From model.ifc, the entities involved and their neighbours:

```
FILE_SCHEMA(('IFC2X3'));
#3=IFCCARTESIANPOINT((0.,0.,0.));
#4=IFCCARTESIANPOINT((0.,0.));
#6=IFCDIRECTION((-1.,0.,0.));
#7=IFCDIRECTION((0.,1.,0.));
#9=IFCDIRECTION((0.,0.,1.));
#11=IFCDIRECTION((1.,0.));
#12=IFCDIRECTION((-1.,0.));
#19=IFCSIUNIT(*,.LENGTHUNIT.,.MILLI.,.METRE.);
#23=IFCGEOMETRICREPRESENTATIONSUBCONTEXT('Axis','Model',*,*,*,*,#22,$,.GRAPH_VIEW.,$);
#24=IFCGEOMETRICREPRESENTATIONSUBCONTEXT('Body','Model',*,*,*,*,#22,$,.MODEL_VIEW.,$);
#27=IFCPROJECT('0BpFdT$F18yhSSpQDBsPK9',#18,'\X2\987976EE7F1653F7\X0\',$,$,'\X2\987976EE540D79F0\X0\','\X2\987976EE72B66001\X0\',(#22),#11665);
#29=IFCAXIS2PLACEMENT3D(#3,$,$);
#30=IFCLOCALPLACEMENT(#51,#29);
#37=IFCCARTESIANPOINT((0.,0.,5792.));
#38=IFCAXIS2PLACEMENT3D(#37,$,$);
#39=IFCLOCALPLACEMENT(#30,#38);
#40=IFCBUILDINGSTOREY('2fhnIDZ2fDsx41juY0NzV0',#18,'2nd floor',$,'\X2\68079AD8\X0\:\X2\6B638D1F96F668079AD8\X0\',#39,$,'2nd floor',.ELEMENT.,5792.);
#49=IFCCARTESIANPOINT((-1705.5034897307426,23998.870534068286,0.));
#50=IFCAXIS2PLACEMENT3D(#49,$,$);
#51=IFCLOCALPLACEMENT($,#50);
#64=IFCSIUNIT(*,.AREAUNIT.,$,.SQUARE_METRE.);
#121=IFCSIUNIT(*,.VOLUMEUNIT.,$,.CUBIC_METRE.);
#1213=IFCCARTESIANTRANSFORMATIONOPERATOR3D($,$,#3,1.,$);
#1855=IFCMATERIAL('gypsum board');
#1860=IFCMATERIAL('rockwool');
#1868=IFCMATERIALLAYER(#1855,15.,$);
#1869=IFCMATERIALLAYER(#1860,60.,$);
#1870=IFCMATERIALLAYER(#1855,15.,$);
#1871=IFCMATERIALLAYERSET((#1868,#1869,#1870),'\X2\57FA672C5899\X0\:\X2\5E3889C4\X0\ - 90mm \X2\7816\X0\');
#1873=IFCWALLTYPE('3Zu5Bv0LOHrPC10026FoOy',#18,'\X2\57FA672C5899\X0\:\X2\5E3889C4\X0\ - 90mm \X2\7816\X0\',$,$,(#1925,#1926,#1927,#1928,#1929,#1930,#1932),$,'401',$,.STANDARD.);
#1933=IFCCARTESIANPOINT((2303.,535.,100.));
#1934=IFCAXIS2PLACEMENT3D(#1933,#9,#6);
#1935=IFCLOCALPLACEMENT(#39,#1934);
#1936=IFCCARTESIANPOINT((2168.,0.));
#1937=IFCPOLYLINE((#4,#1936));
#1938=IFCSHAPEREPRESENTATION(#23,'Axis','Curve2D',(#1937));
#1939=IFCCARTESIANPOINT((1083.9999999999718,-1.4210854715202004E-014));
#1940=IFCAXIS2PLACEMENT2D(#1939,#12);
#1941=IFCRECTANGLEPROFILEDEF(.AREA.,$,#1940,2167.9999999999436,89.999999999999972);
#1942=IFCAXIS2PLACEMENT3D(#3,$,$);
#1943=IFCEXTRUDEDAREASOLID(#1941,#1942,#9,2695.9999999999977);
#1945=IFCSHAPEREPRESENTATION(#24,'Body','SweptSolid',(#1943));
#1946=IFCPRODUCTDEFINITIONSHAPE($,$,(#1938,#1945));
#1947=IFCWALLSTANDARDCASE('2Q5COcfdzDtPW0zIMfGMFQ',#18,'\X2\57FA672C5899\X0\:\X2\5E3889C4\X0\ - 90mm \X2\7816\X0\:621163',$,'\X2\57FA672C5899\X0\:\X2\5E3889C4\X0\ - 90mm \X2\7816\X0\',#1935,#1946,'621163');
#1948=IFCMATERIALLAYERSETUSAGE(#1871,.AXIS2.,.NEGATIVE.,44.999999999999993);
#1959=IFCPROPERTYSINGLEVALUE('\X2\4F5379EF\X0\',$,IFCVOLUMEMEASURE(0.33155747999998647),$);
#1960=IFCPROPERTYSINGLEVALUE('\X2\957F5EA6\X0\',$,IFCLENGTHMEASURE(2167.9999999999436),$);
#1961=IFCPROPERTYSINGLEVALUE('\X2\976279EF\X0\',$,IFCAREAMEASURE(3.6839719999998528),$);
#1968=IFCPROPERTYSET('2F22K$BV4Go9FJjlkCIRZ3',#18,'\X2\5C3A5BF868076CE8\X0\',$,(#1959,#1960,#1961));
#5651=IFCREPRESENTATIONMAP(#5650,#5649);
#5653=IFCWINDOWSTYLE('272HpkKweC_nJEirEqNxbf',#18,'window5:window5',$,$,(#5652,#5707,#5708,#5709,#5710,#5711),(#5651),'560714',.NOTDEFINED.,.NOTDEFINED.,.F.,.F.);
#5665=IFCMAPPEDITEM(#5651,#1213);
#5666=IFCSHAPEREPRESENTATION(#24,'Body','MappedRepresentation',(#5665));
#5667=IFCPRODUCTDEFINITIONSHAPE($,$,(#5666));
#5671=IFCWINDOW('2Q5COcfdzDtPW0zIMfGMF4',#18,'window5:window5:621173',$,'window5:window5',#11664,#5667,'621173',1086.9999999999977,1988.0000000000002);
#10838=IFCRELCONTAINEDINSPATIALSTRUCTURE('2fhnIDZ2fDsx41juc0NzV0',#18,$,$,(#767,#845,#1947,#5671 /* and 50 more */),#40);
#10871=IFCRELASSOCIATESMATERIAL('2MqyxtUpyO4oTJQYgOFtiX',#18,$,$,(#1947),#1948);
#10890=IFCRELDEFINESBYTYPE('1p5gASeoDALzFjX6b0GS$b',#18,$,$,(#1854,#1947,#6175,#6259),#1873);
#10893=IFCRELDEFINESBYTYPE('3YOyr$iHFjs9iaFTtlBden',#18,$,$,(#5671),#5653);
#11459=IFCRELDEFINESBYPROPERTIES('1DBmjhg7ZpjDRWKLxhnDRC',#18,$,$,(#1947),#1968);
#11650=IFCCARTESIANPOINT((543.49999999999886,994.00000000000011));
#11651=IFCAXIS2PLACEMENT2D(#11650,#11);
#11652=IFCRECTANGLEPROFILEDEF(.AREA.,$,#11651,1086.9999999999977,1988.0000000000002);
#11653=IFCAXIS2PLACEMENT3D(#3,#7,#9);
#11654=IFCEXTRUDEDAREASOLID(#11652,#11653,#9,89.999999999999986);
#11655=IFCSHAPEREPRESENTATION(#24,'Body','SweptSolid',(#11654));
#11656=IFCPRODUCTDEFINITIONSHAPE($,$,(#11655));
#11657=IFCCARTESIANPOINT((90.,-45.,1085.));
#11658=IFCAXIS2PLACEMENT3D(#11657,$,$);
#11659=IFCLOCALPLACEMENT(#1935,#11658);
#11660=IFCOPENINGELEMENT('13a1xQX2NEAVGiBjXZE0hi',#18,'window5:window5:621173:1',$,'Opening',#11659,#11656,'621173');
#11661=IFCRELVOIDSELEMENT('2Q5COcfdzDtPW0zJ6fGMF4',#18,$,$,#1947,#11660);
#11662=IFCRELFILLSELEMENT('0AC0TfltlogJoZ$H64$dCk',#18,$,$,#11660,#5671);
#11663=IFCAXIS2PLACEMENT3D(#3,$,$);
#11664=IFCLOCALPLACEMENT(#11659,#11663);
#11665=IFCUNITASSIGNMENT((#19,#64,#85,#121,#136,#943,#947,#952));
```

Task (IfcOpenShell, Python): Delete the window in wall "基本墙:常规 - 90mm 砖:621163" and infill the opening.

```python
import ifcopenshell
import ifcopenshell.api.feature
import ifcopenshell.api.pset
import ifcopenshell.api.root
import ifcopenshell.geom
import ifcopenshell.util.element
import ifcopenshell.util.shape
import ifcopenshell.util.unit

model = ifcopenshell.open("model.ifc")
area_scale = ifcopenshell.util.unit.calculate_unit_scale(model, "AREAUNIT")
volume_scale = ifcopenshell.util.unit.calculate_unit_scale(model, "VOLUMEUNIT")
settings = ifcopenshell.geom.settings()


def volume(element):
    """Net volume in cubic metres, openings subtracted."""
    shape = ifcopenshell.geom.create_shape(settings, element)
    return ifcopenshell.util.shape.get_volume(shape.geometry)


window = model.by_guid("2Q5COcfdzDtPW0zIMfGMF4")
opening = window.FillsVoids[0].RelatingOpeningElement
wall = opening.VoidsElements[0].RelatingBuildingElement
before = volume(wall)

ifcopenshell.api.root.remove_product(model, product=window)
ifcopenshell.api.feature.remove_feature(model, feature=opening)

after = volume(wall)
thickness = 0.09  # wall thickness in metres

# Update the wall's stored quantities.
pset = model.by_id(ifcopenshell.util.element.get_pset(wall, "尺寸标注", should_inherit=False)["id"])
ifcopenshell.api.pset.edit_pset(model, pset=pset, properties={
    "体积": model.create_entity("IfcVolumeMeasure", after / volume_scale),
    "面积": model.create_entity("IfcAreaMeasure", after / thickness / area_scale),
})

print(f"wall volume {before:.3f} -> {after:.3f} m3")

model.write("model_edited.ifc")
```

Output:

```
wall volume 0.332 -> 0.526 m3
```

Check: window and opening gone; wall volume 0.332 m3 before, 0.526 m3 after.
